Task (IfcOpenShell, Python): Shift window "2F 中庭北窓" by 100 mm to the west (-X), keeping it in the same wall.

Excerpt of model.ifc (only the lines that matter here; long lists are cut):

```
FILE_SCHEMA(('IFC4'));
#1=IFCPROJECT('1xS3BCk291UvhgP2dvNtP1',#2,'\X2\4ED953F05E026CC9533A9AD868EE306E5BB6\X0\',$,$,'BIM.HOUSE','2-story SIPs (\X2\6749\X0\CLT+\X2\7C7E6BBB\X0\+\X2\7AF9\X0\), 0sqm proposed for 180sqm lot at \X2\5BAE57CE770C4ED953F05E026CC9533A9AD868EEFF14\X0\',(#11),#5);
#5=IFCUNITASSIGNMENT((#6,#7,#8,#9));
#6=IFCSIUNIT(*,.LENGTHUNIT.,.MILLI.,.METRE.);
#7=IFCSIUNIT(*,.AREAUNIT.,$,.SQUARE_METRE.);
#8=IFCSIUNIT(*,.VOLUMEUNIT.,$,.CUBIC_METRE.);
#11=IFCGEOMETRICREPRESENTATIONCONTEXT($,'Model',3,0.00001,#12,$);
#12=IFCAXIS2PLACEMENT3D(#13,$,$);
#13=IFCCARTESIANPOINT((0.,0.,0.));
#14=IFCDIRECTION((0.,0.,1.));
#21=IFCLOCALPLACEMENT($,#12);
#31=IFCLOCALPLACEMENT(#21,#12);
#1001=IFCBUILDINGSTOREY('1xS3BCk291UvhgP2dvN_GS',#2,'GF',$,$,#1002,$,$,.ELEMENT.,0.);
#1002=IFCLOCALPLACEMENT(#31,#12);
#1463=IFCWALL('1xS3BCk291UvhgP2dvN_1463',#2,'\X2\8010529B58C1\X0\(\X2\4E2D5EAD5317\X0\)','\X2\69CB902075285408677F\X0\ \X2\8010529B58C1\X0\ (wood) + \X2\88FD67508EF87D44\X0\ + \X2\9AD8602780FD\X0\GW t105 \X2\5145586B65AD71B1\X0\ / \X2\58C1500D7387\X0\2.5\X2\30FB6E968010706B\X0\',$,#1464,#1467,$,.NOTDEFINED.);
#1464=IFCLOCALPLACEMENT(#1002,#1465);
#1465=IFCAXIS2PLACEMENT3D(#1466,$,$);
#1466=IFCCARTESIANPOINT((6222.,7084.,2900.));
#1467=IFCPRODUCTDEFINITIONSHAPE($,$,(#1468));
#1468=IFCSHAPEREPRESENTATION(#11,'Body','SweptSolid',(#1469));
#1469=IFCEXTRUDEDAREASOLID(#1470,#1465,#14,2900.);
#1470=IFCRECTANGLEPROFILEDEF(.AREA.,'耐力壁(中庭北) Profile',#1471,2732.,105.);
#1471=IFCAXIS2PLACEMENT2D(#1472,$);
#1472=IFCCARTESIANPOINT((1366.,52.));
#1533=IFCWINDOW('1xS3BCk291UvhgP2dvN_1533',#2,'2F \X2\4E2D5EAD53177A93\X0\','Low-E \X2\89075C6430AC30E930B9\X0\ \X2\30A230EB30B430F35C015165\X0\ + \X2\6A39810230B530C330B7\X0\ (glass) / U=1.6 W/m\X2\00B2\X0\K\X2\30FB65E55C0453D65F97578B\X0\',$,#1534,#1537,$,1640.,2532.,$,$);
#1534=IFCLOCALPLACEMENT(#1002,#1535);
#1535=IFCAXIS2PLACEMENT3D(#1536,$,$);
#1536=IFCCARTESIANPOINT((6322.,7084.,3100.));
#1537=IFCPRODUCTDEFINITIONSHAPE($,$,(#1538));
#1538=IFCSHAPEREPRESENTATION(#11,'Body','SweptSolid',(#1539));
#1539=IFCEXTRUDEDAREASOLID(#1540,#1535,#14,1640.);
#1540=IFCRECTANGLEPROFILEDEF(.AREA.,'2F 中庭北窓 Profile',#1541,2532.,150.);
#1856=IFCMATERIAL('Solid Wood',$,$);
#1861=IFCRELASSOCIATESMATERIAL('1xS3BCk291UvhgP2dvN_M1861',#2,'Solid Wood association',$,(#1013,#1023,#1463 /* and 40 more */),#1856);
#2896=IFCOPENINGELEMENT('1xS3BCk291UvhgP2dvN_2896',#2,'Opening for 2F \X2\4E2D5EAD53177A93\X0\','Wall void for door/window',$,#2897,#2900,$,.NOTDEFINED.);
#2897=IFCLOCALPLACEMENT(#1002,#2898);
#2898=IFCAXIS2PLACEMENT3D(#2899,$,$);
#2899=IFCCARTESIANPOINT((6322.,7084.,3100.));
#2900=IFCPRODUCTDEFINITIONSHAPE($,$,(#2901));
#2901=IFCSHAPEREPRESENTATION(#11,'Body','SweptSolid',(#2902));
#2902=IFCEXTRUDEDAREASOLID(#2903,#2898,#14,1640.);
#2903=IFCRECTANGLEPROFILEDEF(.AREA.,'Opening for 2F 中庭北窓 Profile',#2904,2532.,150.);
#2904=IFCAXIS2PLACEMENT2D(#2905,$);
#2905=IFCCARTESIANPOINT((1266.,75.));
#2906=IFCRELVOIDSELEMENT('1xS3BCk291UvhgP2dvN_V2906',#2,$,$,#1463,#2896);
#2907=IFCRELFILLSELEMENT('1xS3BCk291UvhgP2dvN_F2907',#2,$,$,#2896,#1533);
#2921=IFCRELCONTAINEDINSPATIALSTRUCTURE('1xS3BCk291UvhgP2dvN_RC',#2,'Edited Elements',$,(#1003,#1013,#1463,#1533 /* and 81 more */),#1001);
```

```python
import ifcopenshell
import ifcopenshell.api.geometry
import ifcopenshell.util.placement
import ifcopenshell.util.unit

model = ifcopenshell.open("model.ifc")
unit_scale = ifcopenshell.util.unit.calculate_unit_scale(model)

window = model.by_guid("1xS3BCk291UvhgP2dvN_1533")
opening = window.FillsVoids[0].RelatingOpeningElement
wall = opening.VoidsElements[0].RelatingBuildingElement

wall_matrix = ifcopenshell.util.placement.get_local_placement(wall.ObjectPlacement)
shift = wall_matrix[:3, 0] * -0.1 / unit_scale
before = ifcopenshell.util.placement.get_local_placement(window.ObjectPlacement)[:3, 3].copy()

# The window is not placed relative to its opening, so move both.
for product in (opening, window):
    matrix = ifcopenshell.util.placement.get_local_placement(product.ObjectPlacement)
    matrix[:3, 3] += shift
    ifcopenshell.api.geometry.edit_object_placement(model, product=product, matrix=matrix, is_si=False)

after = ifcopenshell.util.placement.get_local_placement(window.ObjectPlacement)[:3, 3]
print("window moved by", (after - before).round(3) + 0.0)

model.write("model_v2.ifc")
```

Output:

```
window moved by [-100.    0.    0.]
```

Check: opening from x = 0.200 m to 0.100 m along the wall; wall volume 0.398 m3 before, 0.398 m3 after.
